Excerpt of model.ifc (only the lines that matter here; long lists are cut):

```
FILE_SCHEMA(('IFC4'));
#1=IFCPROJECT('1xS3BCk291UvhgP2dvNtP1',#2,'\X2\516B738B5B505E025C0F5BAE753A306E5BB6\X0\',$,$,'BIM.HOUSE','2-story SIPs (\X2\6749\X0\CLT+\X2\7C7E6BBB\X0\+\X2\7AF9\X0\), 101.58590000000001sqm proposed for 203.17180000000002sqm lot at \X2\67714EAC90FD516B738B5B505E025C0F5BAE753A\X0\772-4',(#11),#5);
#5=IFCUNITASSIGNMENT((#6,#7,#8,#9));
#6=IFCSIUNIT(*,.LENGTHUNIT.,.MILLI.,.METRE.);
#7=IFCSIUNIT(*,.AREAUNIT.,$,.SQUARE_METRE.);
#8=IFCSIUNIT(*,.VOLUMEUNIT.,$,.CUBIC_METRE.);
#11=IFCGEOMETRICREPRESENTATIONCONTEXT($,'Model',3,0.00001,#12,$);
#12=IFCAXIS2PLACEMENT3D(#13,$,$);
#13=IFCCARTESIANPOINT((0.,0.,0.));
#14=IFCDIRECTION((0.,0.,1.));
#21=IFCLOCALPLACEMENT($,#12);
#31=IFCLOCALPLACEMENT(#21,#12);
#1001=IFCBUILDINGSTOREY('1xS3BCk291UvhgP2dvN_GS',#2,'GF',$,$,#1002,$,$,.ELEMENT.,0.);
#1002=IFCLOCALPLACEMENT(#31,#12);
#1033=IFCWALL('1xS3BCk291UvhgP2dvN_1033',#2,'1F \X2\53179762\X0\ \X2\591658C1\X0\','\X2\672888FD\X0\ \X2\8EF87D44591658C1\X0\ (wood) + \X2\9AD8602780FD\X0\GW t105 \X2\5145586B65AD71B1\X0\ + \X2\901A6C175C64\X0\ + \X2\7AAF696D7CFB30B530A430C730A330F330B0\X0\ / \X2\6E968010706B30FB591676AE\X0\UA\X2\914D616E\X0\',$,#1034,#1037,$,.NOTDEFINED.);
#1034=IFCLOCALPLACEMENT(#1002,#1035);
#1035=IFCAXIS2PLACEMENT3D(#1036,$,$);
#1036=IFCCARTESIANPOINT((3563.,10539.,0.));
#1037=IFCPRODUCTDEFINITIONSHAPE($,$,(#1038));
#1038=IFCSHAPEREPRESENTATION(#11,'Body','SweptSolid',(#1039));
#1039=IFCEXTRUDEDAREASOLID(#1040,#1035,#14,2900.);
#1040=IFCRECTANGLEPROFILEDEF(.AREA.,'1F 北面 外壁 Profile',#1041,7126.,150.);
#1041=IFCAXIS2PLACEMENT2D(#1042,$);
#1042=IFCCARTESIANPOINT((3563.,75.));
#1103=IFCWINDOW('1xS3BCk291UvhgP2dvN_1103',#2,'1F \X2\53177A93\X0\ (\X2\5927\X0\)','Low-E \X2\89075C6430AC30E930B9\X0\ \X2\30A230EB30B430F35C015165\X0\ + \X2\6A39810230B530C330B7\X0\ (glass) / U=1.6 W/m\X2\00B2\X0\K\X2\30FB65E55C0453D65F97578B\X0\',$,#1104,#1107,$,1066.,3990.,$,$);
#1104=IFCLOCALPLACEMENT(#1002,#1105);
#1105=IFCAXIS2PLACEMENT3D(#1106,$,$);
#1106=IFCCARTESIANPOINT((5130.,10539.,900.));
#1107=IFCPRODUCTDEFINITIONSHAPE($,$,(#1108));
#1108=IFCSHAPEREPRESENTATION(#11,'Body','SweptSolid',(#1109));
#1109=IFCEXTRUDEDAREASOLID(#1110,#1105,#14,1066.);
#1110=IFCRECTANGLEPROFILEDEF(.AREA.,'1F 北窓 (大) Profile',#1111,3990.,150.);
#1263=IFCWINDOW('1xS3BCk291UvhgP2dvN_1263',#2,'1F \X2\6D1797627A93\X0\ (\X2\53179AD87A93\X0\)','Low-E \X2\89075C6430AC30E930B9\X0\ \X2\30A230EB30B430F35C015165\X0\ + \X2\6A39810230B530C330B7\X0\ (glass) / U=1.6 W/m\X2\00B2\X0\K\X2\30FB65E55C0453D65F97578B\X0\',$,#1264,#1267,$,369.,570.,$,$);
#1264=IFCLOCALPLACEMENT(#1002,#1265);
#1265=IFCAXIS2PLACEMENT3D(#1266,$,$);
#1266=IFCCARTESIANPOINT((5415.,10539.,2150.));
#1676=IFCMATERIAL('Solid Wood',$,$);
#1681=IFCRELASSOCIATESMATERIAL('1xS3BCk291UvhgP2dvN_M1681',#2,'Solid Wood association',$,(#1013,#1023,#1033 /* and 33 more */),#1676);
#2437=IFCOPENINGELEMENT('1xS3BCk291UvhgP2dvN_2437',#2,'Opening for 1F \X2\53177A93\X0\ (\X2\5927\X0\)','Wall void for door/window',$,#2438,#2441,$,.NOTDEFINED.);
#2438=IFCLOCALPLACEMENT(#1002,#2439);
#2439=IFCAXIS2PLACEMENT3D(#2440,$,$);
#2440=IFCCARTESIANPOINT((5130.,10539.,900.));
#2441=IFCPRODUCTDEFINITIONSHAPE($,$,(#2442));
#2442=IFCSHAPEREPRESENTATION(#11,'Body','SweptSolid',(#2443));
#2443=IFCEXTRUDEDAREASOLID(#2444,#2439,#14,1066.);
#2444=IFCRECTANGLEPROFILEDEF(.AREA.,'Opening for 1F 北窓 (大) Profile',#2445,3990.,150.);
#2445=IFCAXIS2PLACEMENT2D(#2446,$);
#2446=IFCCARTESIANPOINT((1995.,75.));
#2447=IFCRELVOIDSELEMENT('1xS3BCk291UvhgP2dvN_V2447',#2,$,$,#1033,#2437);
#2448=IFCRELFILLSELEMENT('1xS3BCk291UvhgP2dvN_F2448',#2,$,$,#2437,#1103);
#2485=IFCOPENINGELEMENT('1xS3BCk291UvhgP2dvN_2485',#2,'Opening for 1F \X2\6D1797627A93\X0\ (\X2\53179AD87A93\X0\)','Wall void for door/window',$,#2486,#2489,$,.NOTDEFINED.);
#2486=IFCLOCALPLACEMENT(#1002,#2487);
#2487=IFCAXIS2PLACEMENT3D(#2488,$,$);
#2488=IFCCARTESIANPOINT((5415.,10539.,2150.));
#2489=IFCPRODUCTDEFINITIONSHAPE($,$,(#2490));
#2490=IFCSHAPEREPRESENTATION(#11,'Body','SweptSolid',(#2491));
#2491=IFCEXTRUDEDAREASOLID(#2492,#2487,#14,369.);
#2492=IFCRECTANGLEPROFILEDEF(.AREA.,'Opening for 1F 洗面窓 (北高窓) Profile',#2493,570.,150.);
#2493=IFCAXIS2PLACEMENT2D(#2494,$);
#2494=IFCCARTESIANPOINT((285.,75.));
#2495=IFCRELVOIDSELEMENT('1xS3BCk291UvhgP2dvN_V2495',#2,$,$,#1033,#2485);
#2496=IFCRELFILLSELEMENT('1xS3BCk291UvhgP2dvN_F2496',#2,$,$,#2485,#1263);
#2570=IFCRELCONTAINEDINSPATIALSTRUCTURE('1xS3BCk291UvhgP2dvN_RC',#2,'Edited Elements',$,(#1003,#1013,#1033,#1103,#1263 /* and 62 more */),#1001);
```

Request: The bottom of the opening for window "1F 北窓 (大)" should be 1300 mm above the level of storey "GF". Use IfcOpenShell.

```python
import numpy as np
import ifcopenshell
import ifcopenshell.api.geometry
import ifcopenshell.geom
import ifcopenshell.util.element
import ifcopenshell.util.placement
import ifcopenshell.util.shape
import ifcopenshell.util.unit

model = ifcopenshell.open("model.ifc")
unit_scale = ifcopenshell.util.unit.calculate_unit_scale(model)

window = model.by_guid("1xS3BCk291UvhgP2dvN_1103")
opening = window.FillsVoids[0].RelatingOpeningElement
storey = ifcopenshell.util.element.get_container(window, ifc_class="IfcBuildingStorey")
level = ifcopenshell.util.placement.get_local_placement(storey.ObjectPlacement)[2, 3]

# The opening's origin need not be at the sill, so measure its lowest point.
shape = ifcopenshell.geom.create_shape(ifcopenshell.geom.settings(), opening)
bottom = ifcopenshell.util.shape.get_shape_bottom_elevation(shape, shape.geometry) / unit_scale
dz = level + 1.3 / unit_scale - bottom

shift = np.array([0.0, 0.0, dz])
# The window is not placed relative to its opening, so move both.
for product in (opening, window):
    matrix = ifcopenshell.util.placement.get_local_placement(product.ObjectPlacement)
    matrix[:3, 3] += shift
    ifcopenshell.api.geometry.edit_object_placement(model, product=product, matrix=matrix, is_si=False)

print(f"moved by {dz * unit_scale:+.3f} m")

model.write("model_v2.ifc")
```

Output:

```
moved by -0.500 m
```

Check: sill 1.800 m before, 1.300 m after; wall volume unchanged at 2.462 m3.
